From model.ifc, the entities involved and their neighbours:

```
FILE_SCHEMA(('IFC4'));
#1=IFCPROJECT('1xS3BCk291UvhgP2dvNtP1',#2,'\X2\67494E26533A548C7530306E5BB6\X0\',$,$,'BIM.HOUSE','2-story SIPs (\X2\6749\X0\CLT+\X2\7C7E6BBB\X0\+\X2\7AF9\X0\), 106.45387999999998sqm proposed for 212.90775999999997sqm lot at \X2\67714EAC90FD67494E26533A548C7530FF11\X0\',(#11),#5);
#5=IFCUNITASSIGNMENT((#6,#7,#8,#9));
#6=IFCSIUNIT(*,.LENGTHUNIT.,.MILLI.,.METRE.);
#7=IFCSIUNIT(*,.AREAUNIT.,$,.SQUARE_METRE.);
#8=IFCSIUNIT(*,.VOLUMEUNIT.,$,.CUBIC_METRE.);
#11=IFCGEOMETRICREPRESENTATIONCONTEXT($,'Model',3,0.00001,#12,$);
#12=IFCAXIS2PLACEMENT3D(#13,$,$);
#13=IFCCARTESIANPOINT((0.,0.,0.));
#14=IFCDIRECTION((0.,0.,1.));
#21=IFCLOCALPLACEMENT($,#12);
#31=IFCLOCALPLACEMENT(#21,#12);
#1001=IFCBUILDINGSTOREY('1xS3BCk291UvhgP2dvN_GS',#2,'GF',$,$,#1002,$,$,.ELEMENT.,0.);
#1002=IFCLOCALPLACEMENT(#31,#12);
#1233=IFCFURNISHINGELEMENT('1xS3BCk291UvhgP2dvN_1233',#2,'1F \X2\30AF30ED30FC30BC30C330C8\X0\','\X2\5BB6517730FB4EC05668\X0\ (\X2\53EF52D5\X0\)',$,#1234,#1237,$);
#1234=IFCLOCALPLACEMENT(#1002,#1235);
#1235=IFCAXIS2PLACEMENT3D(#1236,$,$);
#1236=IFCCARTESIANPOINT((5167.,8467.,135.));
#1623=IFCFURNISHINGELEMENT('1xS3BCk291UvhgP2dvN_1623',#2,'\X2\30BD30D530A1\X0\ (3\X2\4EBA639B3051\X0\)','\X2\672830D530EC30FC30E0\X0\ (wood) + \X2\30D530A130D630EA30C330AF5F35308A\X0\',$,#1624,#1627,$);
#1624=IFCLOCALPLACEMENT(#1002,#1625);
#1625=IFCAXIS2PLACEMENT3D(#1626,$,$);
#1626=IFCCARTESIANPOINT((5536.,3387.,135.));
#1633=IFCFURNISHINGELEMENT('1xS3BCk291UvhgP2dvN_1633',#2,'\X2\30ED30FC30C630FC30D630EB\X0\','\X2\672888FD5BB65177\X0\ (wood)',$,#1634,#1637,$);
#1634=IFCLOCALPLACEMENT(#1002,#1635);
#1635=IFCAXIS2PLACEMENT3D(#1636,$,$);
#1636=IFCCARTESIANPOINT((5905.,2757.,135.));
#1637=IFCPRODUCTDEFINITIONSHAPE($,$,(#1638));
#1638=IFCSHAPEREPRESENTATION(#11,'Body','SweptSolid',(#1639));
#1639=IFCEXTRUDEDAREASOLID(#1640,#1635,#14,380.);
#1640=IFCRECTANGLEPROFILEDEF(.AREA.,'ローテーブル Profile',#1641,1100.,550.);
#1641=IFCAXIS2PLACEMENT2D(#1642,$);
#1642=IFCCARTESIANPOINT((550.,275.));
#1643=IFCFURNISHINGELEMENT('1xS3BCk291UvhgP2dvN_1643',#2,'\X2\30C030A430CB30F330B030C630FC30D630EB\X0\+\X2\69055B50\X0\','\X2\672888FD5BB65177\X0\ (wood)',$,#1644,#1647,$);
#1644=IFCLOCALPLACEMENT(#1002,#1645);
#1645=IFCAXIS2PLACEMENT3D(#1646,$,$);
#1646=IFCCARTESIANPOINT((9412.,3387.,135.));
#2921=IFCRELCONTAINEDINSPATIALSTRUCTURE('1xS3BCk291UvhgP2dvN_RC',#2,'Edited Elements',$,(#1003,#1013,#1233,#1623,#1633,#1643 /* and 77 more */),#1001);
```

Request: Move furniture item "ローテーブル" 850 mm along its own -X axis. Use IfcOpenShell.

```python
import ifcopenshell
import ifcopenshell.api.geometry
import ifcopenshell.util.placement
import ifcopenshell.util.unit

model = ifcopenshell.open("model.ifc")
unit_scale = ifcopenshell.util.unit.calculate_unit_scale(model)

item = model.by_guid("1xS3BCk291UvhgP2dvN_1633")
matrix = ifcopenshell.util.placement.get_local_placement(item.ObjectPlacement)
matrix[:3, 3] -= matrix[:3, 0] * 0.85 / unit_scale
ifcopenshell.api.geometry.edit_object_placement(model, product=item, matrix=matrix, is_si=False)

print(ifcopenshell.util.placement.get_local_placement(item.ObjectPlacement).round(3) + 0.0)

model.write("model-out.ifc")
```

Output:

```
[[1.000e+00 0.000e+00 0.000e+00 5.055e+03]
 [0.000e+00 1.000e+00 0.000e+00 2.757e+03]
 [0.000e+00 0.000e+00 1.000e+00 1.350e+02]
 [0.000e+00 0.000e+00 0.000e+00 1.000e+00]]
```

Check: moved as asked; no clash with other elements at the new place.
